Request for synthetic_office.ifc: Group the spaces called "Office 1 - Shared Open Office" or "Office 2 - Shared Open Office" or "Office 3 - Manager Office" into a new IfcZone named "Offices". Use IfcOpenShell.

First a look at what the model holds.

```python
import ifcopenshell

model = ifcopenshell.open("synthetic_office.ifc")
print(model.schema)
seen = {}
for space in model.by_type("IfcSpace"):
    seen[space.LongName] = seen.get(space.LongName, 0) + 1
for name, count in sorted(seen.items(), key=str):
    print(count, "x", name)
print("zones:", [z.Name for z in model.by_type("IfcZone")][:20])
```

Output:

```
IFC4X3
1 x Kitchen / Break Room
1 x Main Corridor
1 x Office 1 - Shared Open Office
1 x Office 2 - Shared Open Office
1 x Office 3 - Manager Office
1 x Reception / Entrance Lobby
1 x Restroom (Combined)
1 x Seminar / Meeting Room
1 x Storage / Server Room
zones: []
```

```python
import ifcopenshell
import ifcopenshell.api.group
import ifcopenshell.api.root

model = ifcopenshell.open("synthetic_office.ifc")

names = {"Office 1 - Shared Open Office", "Office 2 - Shared Open Office", "Office 3 - Manager Office"}
spaces = [s for s in model.by_type("IfcSpace") if s.LongName in names]

zone = ifcopenshell.api.root.create_entity(model, ifc_class="IfcZone", name="Offices")
ifcopenshell.api.group.assign_group(model, products=spaces, group=zone)
print(len(spaces), "spaces in", zone.Name)

model.write("synthetic_office_v2.ifc")
```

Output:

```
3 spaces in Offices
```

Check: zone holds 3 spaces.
